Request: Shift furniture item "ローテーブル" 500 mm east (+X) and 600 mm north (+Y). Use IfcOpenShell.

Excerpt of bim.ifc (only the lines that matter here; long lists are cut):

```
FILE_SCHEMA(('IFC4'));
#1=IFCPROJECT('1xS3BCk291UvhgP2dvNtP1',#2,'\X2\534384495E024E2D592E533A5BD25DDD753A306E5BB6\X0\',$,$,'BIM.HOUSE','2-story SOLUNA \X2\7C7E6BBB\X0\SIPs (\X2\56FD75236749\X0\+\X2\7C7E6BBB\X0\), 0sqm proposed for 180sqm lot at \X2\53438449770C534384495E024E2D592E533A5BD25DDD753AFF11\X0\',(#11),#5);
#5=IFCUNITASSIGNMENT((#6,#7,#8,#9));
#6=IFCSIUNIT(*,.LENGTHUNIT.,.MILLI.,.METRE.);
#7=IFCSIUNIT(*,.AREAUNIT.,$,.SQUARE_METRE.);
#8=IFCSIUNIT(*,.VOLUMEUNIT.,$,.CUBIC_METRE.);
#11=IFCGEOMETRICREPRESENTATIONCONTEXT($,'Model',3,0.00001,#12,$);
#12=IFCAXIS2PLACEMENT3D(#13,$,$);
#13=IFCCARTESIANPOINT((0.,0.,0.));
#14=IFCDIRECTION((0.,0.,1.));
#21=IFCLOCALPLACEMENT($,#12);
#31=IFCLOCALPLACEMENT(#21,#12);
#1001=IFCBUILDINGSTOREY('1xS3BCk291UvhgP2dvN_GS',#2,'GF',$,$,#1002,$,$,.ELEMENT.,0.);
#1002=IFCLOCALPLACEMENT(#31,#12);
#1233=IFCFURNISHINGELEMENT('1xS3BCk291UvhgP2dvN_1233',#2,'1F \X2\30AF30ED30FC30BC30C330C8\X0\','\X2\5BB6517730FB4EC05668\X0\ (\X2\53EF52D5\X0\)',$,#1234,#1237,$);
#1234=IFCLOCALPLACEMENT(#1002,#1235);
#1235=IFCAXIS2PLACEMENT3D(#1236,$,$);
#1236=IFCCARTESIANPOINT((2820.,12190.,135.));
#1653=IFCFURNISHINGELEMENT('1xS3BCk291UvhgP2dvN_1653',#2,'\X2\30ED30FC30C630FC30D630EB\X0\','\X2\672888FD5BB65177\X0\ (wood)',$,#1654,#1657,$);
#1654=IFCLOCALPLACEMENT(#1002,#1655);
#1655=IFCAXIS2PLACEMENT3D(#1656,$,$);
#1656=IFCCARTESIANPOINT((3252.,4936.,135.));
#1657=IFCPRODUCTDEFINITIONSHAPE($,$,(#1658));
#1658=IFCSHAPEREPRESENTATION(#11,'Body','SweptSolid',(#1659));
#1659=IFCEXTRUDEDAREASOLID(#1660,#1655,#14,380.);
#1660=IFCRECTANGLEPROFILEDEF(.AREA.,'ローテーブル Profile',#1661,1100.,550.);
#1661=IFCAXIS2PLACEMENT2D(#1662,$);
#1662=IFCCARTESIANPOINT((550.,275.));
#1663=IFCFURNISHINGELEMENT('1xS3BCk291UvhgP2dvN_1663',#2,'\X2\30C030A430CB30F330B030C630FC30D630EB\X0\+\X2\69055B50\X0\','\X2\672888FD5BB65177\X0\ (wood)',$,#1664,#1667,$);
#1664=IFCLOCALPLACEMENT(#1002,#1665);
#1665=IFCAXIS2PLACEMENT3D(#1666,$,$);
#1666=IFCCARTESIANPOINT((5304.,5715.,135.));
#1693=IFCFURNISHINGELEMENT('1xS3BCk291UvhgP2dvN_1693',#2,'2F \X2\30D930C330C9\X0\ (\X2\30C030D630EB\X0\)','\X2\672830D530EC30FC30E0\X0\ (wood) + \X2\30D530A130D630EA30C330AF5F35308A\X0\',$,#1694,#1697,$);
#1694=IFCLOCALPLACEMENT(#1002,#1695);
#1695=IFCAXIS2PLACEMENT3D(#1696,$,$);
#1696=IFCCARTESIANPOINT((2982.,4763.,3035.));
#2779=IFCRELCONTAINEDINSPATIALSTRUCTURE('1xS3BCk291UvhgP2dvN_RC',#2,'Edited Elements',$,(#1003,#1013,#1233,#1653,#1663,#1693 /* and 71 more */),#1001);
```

```python
import ifcopenshell
import ifcopenshell.api.geometry
import ifcopenshell.util.placement
import ifcopenshell.util.unit

model = ifcopenshell.open("bim.ifc")
unit_scale = ifcopenshell.util.unit.calculate_unit_scale(model)

item = model.by_id(1653)
matrix = ifcopenshell.util.placement.get_local_placement(item.ObjectPlacement)
matrix[0, 3] += 0.5 / unit_scale
matrix[1, 3] += 0.6 / unit_scale
ifcopenshell.api.geometry.edit_object_placement(model, product=item, matrix=matrix, is_si=False)

print(ifcopenshell.util.placement.get_local_placement(item.ObjectPlacement).round(3) + 0.0)

model.write("bim-out.ifc")
```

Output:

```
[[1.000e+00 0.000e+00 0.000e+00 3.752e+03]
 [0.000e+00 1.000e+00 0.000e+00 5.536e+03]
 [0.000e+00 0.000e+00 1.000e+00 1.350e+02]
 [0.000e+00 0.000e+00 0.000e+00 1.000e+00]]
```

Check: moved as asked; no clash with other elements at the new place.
